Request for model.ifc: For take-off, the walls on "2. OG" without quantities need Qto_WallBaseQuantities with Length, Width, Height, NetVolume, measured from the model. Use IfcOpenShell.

First a look at what the model holds.

```python
import ifcopenshell
import ifcopenshell.util.element
import ifcopenshell.util.unit

model = ifcopenshell.open("model.ifc")
print(model.schema)
for unit_type in ("LENGTHUNIT", "AREAUNIT", "VOLUMEUNIT"):
    print(unit_type, ifcopenshell.util.unit.calculate_unit_scale(model, unit_type))
storey = next(s for s in model.by_type("IfcBuildingStorey") if s.Name == "2. OG")
walls = [e for e in ifcopenshell.util.element.get_decomposition(storey) if e.is_a("IfcWall")]
for e in sorted(walls, key=lambda e: e.id()):
    print(e.id(), e.is_a(), e.Name, list(ifcopenshell.util.element.get_psets(e, qtos_only=True)), sep=" | ")
```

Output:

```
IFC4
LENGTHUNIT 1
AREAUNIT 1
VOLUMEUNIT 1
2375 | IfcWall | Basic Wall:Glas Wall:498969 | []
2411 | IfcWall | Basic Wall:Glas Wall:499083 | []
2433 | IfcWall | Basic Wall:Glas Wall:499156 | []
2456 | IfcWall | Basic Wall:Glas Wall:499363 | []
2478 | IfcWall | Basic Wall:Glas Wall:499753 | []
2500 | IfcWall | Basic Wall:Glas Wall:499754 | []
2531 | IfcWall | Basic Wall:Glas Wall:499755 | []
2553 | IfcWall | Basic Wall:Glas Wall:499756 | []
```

```python
import ifcopenshell
import ifcopenshell.api.pset
import ifcopenshell.geom
import ifcopenshell.util.element
import ifcopenshell.util.shape
import ifcopenshell.util.unit

model = ifcopenshell.open("model.ifc")
unit_scale = ifcopenshell.util.unit.calculate_unit_scale(model)
volume_scale = ifcopenshell.util.unit.calculate_unit_scale(model, "VOLUMEUNIT")
settings = ifcopenshell.geom.settings()

storey = next(s for s in model.by_type("IfcBuildingStorey") if s.Name == "2. OG")
walls = [e for e in ifcopenshell.util.element.get_decomposition(storey) if e.is_a("IfcWall")]

for e in sorted(walls, key=lambda e: e.id()):
    if ifcopenshell.util.element.get_psets(e, qtos_only=True, should_inherit=False):
        continue
    # Geometry comes back in metres, in the element's own axes.
    shape = ifcopenshell.geom.create_shape(settings, e)
    values = {
        "Length": ifcopenshell.util.shape.get_x(shape.geometry) / unit_scale,
        "Width": ifcopenshell.util.shape.get_y(shape.geometry) / unit_scale,
        "Height": ifcopenshell.util.shape.get_z(shape.geometry) / unit_scale,
        "NetVolume": ifcopenshell.util.shape.get_volume(shape.geometry) / volume_scale,
    }
    qto = ifcopenshell.api.pset.add_qto(model, product=e, name="Qto_WallBaseQuantities")
    ifcopenshell.api.pset.edit_qto(model, qto=qto, properties=values)
    print(e.id(), {k: round(v, 3) for k, v in values.items()})

model.write("model_rev.ifc")
```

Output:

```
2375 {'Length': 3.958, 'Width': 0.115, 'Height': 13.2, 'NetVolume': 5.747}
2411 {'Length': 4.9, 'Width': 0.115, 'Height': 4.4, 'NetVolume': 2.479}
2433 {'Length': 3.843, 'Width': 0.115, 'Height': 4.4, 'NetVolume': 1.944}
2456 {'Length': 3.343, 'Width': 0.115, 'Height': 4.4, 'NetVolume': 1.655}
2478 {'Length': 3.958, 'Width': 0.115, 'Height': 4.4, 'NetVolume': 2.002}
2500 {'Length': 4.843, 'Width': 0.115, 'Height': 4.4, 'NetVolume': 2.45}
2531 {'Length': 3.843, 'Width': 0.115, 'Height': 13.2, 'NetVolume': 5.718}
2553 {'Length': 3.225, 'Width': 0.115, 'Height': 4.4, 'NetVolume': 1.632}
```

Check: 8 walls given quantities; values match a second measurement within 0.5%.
